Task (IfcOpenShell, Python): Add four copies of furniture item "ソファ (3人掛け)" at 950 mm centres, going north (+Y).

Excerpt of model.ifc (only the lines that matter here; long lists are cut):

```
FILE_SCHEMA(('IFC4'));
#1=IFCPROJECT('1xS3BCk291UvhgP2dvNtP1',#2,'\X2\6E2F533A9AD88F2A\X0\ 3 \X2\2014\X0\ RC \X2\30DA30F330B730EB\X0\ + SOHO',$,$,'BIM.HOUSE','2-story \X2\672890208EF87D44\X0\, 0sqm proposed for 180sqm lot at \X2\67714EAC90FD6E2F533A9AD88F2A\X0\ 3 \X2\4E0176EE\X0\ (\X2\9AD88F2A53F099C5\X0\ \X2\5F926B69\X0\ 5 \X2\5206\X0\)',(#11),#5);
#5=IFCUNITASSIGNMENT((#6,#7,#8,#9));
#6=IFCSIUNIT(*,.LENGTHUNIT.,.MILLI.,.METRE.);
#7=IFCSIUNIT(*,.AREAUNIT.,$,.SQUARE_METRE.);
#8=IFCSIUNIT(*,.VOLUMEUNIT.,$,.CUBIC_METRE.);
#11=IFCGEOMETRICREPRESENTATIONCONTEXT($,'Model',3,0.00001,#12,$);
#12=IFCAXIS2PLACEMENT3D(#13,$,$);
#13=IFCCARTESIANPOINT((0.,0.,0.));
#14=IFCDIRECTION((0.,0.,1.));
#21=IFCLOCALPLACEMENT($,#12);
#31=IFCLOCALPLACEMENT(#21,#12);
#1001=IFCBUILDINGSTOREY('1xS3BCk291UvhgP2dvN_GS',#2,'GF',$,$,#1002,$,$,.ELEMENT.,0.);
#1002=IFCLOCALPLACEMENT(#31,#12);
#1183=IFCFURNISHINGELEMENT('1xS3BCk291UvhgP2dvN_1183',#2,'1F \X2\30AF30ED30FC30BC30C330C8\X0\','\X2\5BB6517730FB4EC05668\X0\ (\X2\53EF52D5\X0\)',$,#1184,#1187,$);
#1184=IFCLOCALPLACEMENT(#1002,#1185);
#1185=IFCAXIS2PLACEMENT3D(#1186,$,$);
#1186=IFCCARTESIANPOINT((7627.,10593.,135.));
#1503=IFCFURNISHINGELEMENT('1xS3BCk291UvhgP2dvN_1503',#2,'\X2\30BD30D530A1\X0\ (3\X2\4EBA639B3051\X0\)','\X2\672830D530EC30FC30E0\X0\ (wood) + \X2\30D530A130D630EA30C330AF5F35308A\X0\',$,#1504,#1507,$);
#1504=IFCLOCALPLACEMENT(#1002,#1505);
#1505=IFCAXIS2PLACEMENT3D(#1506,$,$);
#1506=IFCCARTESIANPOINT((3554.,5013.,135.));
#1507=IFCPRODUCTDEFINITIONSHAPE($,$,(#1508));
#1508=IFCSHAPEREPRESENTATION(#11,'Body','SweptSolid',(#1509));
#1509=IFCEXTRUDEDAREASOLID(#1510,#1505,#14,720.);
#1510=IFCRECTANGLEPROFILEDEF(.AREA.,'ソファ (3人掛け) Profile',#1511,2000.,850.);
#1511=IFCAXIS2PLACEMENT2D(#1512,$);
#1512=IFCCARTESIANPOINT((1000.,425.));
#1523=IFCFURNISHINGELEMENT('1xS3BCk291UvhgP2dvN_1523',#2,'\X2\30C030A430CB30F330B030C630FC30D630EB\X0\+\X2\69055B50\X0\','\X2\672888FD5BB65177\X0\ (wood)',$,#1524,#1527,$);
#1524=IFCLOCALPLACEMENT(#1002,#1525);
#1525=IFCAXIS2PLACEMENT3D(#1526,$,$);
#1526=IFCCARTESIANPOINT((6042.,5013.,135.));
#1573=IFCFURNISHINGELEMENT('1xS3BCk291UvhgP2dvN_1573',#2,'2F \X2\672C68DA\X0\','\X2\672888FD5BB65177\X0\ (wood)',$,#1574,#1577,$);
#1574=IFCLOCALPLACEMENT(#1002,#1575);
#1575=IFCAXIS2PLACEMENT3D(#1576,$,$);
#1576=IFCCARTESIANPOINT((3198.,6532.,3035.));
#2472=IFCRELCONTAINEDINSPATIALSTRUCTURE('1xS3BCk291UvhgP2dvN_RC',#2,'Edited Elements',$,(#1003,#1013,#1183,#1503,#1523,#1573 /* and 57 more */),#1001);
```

```python
import numpy as np
import ifcopenshell
import ifcopenshell.api.geometry
import ifcopenshell.api.root
import ifcopenshell.util.element
import ifcopenshell.util.placement

model = ifcopenshell.open("model.ifc")


def reuse_history(source, copy):
    """copy_class also copies each property set's owner history, people and application; keep the originals."""
    for rel in copy.IsDefinedBy:
        if rel.is_a("IfcRelDefinesByProperties") and (history := rel.RelatingPropertyDefinition.OwnerHistory):
            rel.RelatingPropertyDefinition.OwnerHistory = source.OwnerHistory
            ifcopenshell.util.element.remove_deep2(model, history)


source = model.by_id(1503)
base = ifcopenshell.util.placement.get_local_placement(source.ObjectPlacement)
step = np.array([0.0, 1.0, 0.0]) * 950.0

for i in range(1, 5):
    copy = ifcopenshell.api.root.copy_class(model, product=source)
    copy.Representation = ifcopenshell.util.element.copy_deep(
        model, source.Representation, exclude=["IfcGeometricRepresentationContext", "IfcRepresentationMap"]
    )
    reuse_history(source, copy)
    matrix = base.copy()
    matrix[:3, 3] += i * step
    print("added at", matrix[:3, 3].round(3) + 0.0)
    ifcopenshell.api.geometry.edit_object_placement(model, product=copy, matrix=matrix, is_si=False)

model.write("model-out.ifc")
```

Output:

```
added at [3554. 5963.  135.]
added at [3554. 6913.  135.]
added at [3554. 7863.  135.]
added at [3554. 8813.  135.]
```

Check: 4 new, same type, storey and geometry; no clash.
